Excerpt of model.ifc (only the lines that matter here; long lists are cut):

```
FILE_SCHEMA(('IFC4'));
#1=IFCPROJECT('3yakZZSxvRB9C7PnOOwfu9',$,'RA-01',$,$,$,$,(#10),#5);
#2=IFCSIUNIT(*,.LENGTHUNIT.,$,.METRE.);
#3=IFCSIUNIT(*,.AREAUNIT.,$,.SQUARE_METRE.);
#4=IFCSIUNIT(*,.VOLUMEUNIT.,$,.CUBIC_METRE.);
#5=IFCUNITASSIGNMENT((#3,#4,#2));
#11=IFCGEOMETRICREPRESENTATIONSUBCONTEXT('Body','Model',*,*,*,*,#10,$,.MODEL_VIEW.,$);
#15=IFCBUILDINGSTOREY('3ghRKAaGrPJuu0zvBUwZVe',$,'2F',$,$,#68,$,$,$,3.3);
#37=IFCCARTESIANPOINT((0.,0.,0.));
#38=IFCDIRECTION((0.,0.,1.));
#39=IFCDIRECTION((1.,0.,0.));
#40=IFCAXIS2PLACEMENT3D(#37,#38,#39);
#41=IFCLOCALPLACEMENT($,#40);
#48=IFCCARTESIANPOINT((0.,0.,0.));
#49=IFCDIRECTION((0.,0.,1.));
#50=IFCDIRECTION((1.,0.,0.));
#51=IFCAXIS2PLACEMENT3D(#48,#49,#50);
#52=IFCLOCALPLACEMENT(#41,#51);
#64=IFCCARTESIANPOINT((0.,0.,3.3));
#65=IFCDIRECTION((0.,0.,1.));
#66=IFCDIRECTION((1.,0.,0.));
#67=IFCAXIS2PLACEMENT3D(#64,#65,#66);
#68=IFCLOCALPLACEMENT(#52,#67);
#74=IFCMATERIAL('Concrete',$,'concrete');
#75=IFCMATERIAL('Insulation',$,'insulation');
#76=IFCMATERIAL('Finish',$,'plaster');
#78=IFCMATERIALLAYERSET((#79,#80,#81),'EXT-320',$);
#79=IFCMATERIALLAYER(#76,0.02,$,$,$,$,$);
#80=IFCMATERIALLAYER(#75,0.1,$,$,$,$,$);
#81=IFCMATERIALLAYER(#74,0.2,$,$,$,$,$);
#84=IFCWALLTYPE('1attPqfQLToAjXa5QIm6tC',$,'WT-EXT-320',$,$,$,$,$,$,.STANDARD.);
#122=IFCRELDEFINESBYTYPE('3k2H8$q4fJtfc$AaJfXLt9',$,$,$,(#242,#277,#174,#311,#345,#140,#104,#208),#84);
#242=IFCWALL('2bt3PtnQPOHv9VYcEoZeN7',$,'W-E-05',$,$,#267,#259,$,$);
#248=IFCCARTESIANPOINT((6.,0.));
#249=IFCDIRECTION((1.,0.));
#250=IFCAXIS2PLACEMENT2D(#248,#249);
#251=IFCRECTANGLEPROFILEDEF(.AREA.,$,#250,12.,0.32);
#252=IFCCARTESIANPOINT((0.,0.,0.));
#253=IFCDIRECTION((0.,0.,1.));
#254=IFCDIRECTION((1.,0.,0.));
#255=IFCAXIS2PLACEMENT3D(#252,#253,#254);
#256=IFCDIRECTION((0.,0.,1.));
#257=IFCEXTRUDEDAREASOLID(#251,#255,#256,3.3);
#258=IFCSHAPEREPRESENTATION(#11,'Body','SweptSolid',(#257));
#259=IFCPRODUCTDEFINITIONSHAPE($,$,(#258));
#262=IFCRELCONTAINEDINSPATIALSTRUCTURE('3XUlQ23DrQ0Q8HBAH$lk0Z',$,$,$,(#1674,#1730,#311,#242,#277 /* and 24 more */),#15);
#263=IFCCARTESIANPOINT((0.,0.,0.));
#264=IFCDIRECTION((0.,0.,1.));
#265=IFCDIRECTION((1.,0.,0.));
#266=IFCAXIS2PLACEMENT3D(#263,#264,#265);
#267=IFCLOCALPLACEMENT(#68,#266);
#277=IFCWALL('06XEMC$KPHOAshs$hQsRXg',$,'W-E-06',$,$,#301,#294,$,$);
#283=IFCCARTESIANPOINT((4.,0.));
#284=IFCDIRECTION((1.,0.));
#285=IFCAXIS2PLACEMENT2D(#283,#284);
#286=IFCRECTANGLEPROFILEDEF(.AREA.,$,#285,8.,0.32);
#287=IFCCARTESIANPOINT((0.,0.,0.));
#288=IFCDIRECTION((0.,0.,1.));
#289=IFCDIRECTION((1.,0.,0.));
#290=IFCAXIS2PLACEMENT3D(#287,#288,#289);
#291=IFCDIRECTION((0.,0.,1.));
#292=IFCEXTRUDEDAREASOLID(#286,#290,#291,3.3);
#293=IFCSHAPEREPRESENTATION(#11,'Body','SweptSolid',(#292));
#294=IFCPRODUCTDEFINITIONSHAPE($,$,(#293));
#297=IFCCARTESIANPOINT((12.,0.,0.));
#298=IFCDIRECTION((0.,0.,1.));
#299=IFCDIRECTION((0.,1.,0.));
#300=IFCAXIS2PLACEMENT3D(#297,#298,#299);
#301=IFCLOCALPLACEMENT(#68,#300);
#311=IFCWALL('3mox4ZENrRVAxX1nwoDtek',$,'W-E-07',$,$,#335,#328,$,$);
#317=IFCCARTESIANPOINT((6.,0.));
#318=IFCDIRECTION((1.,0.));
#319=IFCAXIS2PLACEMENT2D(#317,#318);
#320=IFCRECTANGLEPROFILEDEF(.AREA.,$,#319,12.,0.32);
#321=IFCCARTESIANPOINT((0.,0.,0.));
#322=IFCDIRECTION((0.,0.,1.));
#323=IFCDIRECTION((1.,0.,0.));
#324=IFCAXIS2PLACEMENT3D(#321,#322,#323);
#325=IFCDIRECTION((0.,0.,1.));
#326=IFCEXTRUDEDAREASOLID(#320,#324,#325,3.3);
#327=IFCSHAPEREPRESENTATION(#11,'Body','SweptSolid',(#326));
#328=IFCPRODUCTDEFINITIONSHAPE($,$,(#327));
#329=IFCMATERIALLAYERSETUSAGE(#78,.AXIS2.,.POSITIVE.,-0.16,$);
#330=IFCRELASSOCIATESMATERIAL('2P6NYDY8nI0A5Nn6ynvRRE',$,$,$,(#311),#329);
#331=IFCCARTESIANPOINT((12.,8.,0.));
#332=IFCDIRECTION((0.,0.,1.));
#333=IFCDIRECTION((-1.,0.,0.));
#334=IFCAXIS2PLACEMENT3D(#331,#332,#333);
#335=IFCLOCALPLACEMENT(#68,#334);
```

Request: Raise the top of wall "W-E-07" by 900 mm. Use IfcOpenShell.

```python
import ifcopenshell
import ifcopenshell.geom
import ifcopenshell.util.representation
import ifcopenshell.util.shape
import ifcopenshell.util.unit

model = ifcopenshell.open("model.ifc")
unit_scale = ifcopenshell.util.unit.calculate_unit_scale(model)
settings = ifcopenshell.geom.settings()


def volume(element):
    """Net volume in cubic metres, openings subtracted."""
    shape = ifcopenshell.geom.create_shape(settings, element)
    return ifcopenshell.util.shape.get_volume(shape.geometry)


wall = model.by_guid("3mox4ZENrRVAxX1nwoDtek")
before = volume(wall)

body = ifcopenshell.util.representation.get_representation(wall, "Model", "Body")
solid = body.Items[0]
old_height = solid.Depth
solid.Depth += 0.9 / unit_scale
after = volume(wall)

print(f"height {old_height:g} -> {solid.Depth:g}, volume {before:.3f} -> {after:.3f} m3")

model.write("model_edited.ifc")
```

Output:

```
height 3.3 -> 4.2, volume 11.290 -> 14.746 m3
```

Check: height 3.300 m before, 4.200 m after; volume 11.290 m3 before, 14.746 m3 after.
